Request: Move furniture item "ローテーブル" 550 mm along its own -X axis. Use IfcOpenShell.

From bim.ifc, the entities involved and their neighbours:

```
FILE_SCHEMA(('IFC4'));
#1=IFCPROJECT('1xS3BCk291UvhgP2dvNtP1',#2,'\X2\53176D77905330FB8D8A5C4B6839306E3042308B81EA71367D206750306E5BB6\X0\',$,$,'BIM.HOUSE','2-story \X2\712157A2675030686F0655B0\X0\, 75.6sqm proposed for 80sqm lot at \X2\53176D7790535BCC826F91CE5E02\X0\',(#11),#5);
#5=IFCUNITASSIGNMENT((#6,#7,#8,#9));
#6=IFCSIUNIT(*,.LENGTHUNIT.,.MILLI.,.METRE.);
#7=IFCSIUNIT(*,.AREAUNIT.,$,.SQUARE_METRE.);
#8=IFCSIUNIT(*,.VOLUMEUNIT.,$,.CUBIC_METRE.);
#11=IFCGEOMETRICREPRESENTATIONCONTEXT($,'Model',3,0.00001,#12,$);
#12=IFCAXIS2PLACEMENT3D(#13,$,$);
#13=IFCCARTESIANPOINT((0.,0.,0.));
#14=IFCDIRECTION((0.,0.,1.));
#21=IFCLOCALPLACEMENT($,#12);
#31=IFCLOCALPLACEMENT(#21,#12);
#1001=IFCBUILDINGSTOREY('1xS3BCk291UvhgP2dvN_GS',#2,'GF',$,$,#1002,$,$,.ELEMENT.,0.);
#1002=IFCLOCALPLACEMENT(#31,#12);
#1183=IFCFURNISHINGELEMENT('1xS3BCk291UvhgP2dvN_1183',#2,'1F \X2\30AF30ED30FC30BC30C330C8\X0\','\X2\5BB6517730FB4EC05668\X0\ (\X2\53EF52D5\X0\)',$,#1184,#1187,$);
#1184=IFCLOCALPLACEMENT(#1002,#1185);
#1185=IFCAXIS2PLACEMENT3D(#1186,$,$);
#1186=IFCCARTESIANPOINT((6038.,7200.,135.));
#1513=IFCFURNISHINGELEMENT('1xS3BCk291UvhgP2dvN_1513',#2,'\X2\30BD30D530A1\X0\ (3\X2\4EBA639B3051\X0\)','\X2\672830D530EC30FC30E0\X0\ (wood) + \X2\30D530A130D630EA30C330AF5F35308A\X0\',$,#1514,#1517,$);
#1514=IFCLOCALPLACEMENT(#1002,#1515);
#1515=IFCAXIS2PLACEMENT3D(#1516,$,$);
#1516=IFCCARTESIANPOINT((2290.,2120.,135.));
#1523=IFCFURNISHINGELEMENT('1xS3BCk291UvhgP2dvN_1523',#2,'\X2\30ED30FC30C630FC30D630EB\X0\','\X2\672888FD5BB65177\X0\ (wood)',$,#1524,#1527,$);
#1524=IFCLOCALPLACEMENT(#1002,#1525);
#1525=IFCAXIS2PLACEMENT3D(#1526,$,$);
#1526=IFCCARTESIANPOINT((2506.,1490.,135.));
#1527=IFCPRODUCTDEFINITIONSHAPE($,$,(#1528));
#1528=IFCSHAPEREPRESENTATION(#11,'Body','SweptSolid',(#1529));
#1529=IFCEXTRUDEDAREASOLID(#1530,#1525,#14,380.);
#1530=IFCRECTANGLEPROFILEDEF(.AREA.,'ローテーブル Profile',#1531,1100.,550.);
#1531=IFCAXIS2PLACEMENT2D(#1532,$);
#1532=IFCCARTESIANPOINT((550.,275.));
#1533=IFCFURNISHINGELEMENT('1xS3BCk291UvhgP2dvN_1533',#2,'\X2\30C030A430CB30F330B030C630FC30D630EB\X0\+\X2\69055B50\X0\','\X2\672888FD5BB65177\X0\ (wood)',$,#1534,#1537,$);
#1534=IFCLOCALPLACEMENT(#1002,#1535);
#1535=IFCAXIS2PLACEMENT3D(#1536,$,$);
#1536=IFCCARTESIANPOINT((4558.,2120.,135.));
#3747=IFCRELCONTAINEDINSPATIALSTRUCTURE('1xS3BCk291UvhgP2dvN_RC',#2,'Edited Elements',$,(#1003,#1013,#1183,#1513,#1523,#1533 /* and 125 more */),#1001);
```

```python
import ifcopenshell
import ifcopenshell.api.geometry
import ifcopenshell.util.placement
import ifcopenshell.util.unit

model = ifcopenshell.open("bim.ifc")
unit_scale = ifcopenshell.util.unit.calculate_unit_scale(model)

item = model.by_guid("1xS3BCk291UvhgP2dvN_1523")
matrix = ifcopenshell.util.placement.get_local_placement(item.ObjectPlacement)
matrix[:3, 3] -= matrix[:3, 0] * 0.55 / unit_scale
ifcopenshell.api.geometry.edit_object_placement(model, product=item, matrix=matrix, is_si=False)

print(ifcopenshell.util.placement.get_local_placement(item.ObjectPlacement).round(3) + 0.0)

model.write("bim_edited.ifc")
```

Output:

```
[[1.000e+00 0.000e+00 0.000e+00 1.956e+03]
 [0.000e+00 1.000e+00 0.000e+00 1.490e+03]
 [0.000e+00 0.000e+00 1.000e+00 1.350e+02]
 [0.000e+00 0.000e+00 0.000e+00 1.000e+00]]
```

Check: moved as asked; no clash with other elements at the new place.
